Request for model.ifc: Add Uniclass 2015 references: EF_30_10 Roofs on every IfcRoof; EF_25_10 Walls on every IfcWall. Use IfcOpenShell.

First a look at what the model holds.

```python
import ifcopenshell

model = ifcopenshell.open("model.ifc")
print(model.schema)
print("classifications:", [c.Name for c in model.by_type("IfcClassification")])
for ifc_class in ("IfcDoor", "IfcRoof", "IfcStair", "IfcWall", "IfcWindow"):
    print(ifc_class, len(model.by_type(ifc_class)))
```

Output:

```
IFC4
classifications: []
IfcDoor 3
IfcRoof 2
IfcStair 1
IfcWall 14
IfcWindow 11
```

```python
import ifcopenshell
import ifcopenshell.api.classification

model = ifcopenshell.open("model.ifc")

system = ifcopenshell.api.classification.add_classification(model, classification="Uniclass 2015")

codes = {
    "IfcRoof": ("EF_30_10", "Roofs"),
    "IfcWall": ("EF_25_10", "Walls"),
}
for ifc_class, (code, name) in codes.items():
    products = model.by_type(ifc_class)
    ifcopenshell.api.classification.add_reference(
        model, products=products, classification=system, identification=code, name=name
    )
    print(code, len(products))

model.write("model_rev.ifc")
```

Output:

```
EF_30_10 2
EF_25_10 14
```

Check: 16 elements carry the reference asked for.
